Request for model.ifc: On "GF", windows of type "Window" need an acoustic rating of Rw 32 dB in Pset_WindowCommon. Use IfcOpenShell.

First a look at what the model holds.

```python
import ifcopenshell
import ifcopenshell.util.element

model = ifcopenshell.open("model.ifc")
print(model.schema)
storey = next(s for s in model.by_type("IfcBuildingStorey") if s.Name == "GF")
windows = [e for e in ifcopenshell.util.element.get_decomposition(storey) if e.is_a("IfcWindow")]
seen = {}
for e in windows:
    element_type = ifcopenshell.util.element.get_type(e)
    key = (element_type.Name if element_type != e and element_type else None, ifcopenshell.util.element.get_pset(e, "Pset_WindowCommon", "AcousticRating"))
    seen[key] = seen.get(key, 0) + 1
for (name, value), count in sorted(seen.items(), key=str):
    print(count, "x", name, "|", value)
```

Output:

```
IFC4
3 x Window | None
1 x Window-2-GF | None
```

```python
import ifcopenshell
import ifcopenshell.api.pset
import ifcopenshell.util.element

model = ifcopenshell.open("model.ifc")

storey = next(s for s in model.by_type("IfcBuildingStorey") if s.Name == "GF")
windows = [e for e in ifcopenshell.util.element.get_decomposition(storey) if e.is_a("IfcWindow")]

count = 0
for e in windows:
    element_type = ifcopenshell.util.element.get_type(e)
    if element_type in (None, e) or element_type.Name != "Window":
        continue
    # add_pset returns the element's existing set when there is one.
    pset = ifcopenshell.api.pset.add_pset(model, product=e, name="Pset_WindowCommon")
    ifcopenshell.api.pset.edit_pset(model, pset=pset, properties={"AcousticRating": "Rw 32 dB"})
    count += 1

print(count, "windows updated")

model.write("model_updated.ifc")
```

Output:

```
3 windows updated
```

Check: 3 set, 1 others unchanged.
